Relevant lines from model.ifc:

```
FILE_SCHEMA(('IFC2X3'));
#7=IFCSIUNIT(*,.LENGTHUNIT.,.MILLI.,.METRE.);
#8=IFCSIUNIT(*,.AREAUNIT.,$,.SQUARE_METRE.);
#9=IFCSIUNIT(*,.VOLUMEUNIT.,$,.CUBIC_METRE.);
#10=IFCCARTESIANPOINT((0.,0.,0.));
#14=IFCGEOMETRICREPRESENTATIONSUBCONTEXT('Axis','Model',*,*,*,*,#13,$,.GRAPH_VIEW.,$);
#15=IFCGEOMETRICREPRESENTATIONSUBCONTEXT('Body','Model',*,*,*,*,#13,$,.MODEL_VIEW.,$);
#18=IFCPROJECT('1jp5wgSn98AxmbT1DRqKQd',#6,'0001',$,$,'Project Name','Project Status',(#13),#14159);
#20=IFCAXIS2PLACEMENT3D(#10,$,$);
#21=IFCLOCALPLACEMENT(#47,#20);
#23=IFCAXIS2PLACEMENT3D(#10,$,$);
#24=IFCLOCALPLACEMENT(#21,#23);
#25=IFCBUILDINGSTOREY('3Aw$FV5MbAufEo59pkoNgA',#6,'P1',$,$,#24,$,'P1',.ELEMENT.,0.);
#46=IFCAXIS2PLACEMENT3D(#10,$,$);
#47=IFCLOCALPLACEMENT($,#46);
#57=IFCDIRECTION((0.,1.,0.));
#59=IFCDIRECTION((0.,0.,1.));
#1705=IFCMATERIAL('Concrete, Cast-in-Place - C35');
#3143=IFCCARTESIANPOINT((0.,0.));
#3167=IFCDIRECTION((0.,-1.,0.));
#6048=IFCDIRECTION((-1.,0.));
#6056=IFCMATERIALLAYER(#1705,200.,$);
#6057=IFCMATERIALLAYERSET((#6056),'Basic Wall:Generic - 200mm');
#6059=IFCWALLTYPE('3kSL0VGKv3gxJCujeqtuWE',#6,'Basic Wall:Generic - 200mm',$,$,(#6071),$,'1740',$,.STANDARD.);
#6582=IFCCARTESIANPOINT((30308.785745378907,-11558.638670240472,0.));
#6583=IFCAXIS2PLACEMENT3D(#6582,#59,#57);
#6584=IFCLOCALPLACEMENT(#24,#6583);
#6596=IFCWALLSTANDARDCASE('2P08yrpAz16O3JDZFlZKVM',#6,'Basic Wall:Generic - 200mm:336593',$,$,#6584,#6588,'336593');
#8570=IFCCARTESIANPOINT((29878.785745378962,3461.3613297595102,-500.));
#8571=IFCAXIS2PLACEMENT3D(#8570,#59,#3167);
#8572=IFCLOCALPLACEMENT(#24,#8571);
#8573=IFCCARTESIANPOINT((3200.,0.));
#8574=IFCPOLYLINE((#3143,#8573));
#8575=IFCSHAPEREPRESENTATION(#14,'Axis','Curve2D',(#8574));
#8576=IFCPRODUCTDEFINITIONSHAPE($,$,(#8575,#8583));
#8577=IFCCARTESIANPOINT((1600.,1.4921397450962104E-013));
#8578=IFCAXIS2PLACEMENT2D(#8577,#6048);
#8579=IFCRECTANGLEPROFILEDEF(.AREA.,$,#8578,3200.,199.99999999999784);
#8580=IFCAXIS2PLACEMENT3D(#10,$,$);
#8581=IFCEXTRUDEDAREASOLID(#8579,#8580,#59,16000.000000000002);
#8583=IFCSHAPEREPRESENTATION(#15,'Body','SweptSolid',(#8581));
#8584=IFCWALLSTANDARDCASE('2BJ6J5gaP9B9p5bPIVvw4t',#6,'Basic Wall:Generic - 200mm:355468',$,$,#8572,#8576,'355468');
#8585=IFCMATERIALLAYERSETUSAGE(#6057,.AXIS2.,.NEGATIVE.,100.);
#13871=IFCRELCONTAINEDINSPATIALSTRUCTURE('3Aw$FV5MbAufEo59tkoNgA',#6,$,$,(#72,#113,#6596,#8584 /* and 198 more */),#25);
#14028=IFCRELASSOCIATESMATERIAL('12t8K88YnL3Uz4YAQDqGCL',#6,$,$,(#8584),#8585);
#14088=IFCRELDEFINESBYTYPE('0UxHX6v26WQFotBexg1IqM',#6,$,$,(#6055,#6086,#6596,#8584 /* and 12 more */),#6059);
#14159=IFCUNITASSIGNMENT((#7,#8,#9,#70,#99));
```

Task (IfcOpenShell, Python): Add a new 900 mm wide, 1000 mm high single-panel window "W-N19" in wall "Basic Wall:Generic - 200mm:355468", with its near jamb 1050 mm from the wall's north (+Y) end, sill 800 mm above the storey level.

```python
import numpy as np
import ifcopenshell
import ifcopenshell.api.feature
import ifcopenshell.api.geometry
import ifcopenshell.api.root
import ifcopenshell.api.spatial
import ifcopenshell.api.type
import ifcopenshell.geom
import ifcopenshell.util.element
import ifcopenshell.util.placement
import ifcopenshell.util.representation
import ifcopenshell.util.shape
import ifcopenshell.util.unit

model = ifcopenshell.open("model.ifc")
unit_scale = ifcopenshell.util.unit.calculate_unit_scale(model)
settings = ifcopenshell.geom.settings()


def volume(element):
    """Net volume in cubic metres, openings subtracted."""
    shape = ifcopenshell.geom.create_shape(settings, element)
    return ifcopenshell.util.shape.get_volume(shape.geometry)


wall = model.by_guid("2BJ6J5gaP9B9p5bPIVvw4t")
storey = ifcopenshell.util.element.get_container(wall, ifc_class="IfcBuildingStorey")
context = ifcopenshell.util.representation.get_context(model, "Model", "Body", "MODEL_VIEW")
before = volume(wall)

width, height, from_end, sill = 0.9, 1, 1.05, 0.8  # metres

# The wall runs along its own X axis, and the end named is its -X end.
wall_shape = ifcopenshell.geom.create_shape(settings, wall)
x, y, z = ifcopenshell.util.shape.get_vertices(wall_shape.geometry).T
start = x.min() + from_end
face, thickness = float(y.min()), float(y.max() - y.min())
wall_matrix = ifcopenshell.util.placement.get_local_placement(wall.ObjectPlacement)
level = ifcopenshell.util.placement.get_local_placement(storey.ObjectPlacement)[2, 3]


def in_wall(x, y):
    """Placement at x, y metres in the wall's axes, at sill height."""
    matrix = wall_matrix.copy()
    matrix[:, 3] = wall_matrix @ np.array([x / unit_scale, y / unit_scale, 0.0, 1.0])
    matrix[2, 3] = level + sill / unit_scale
    return matrix


# Opening: a box that overshoots both wall faces by 50 mm.
opening = ifcopenshell.api.root.create_entity(model, ifc_class="IfcOpeningElement")
box = ifcopenshell.api.geometry.add_wall_representation(
    model, context=context, length=width, height=height, thickness=thickness + 0.1
)
ifcopenshell.api.geometry.assign_representation(model, product=opening, representation=box)
ifcopenshell.api.geometry.edit_object_placement(model, product=opening, matrix=in_wall(start, face - 0.05), is_si=False)
ifcopenshell.api.feature.add_feature(model, feature=opening, element=wall)

window = ifcopenshell.api.root.create_entity(model, ifc_class="IfcWindow", name="W-N19")
window.OverallWidth, window.OverallHeight = width / unit_scale, height / unit_scale
body = ifcopenshell.api.geometry.add_window_representation(
    model,
    context=context,
    overall_width=window.OverallWidth,
    overall_height=window.OverallHeight,
    partition_type="SINGLE_PANEL",
)
ifcopenshell.api.geometry.assign_representation(model, product=window, representation=body)
ifcopenshell.api.spatial.assign_container(model, products=[window], relating_structure=storey)
fills = ifcopenshell.api.feature.add_filling(model, opening=opening, element=window)
fills.OwnerHistory = window.OwnerHistory  # required in IFC2X3

# IFC2X3 keeps the operation on the window style.
style = ifcopenshell.api.root.create_entity(model, ifc_class="IfcWindowStyle", name="W-N19")
style.OperationType, style.ConstructionType = "SINGLE_PANEL", "NOTDEFINED"
style.ParameterTakesPrecedence = style.Sizeable = False
ifcopenshell.api.type.assign_type(model, related_objects=[window], relating_type=style)

# Centre the window in the wall's thickness.
ifcopenshell.api.geometry.edit_object_placement(model, product=window, matrix=in_wall(start, face), is_si=False)
window_shape = ifcopenshell.geom.create_shape(settings, window)
depth = ifcopenshell.util.shape.get_vertices(window_shape.geometry)[:, 1]
offset = face + thickness / 2 - (depth.min() + depth.max()) / 2
ifcopenshell.api.geometry.edit_object_placement(model, product=window, matrix=in_wall(start, offset), is_si=False)

after = volume(wall)

print(f"wall volume {before:.3f} -> {after:.3f} m3")

model.write("model-out.ifc")
```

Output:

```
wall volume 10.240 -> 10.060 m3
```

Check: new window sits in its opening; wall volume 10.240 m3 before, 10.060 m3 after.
